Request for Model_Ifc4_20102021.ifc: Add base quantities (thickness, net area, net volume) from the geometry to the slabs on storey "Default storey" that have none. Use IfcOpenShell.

First a look at what the model holds.

```python
import ifcopenshell
import ifcopenshell.util.element
import ifcopenshell.util.unit

model = ifcopenshell.open("Model_Ifc4_20102021.ifc")
print(model.schema)
for unit_type in ("LENGTHUNIT", "AREAUNIT", "VOLUMEUNIT"):
    print(unit_type, ifcopenshell.util.unit.calculate_unit_scale(model, unit_type))
storey = next(s for s in model.by_type("IfcBuildingStorey") if s.Name == "Default storey")
slabs = [e for e in ifcopenshell.util.element.get_decomposition(storey) if e.is_a("IfcSlab")]
for e in sorted(slabs, key=lambda e: e.id()):
    print(e.id(), e.is_a(), e.Name, list(ifcopenshell.util.element.get_psets(e, qtos_only=True)), sep=" | ")
```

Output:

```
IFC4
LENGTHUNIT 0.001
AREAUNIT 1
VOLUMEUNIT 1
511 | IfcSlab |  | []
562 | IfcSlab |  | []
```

```python
import ifcopenshell
import ifcopenshell.api.pset
import ifcopenshell.geom
import ifcopenshell.util.element
import ifcopenshell.util.shape
import ifcopenshell.util.unit

model = ifcopenshell.open("Model_Ifc4_20102021.ifc")
unit_scale = ifcopenshell.util.unit.calculate_unit_scale(model)
area_scale = ifcopenshell.util.unit.calculate_unit_scale(model, "AREAUNIT")
volume_scale = ifcopenshell.util.unit.calculate_unit_scale(model, "VOLUMEUNIT")
settings = ifcopenshell.geom.settings()

storey = next(s for s in model.by_type("IfcBuildingStorey") if s.Name == "Default storey")
slabs = [e for e in ifcopenshell.util.element.get_decomposition(storey) if e.is_a("IfcSlab")]

for e in sorted(slabs, key=lambda e: e.id()):
    if ifcopenshell.util.element.get_psets(e, qtos_only=True, should_inherit=False):
        continue
    # Geometry comes back in metres, in the element's own axes.
    shape = ifcopenshell.geom.create_shape(settings, e)
    values = {
        "Width": ifcopenshell.util.shape.get_z(shape.geometry) / unit_scale,
        "NetArea": ifcopenshell.util.shape.get_footprint_area(shape.geometry) / area_scale,
        "NetVolume": ifcopenshell.util.shape.get_volume(shape.geometry) / volume_scale,
    }
    qto = ifcopenshell.api.pset.add_qto(model, product=e, name="Qto_SlabBaseQuantities")
    ifcopenshell.api.pset.edit_qto(model, qto=qto, properties=values)
    print(e.id(), {k: round(v, 3) for k, v in values.items()})

model.write("Model_Ifc4_20102021_updated.ifc")
```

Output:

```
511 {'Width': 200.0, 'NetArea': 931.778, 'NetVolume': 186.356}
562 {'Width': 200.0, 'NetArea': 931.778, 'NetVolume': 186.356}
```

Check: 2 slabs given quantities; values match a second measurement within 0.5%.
